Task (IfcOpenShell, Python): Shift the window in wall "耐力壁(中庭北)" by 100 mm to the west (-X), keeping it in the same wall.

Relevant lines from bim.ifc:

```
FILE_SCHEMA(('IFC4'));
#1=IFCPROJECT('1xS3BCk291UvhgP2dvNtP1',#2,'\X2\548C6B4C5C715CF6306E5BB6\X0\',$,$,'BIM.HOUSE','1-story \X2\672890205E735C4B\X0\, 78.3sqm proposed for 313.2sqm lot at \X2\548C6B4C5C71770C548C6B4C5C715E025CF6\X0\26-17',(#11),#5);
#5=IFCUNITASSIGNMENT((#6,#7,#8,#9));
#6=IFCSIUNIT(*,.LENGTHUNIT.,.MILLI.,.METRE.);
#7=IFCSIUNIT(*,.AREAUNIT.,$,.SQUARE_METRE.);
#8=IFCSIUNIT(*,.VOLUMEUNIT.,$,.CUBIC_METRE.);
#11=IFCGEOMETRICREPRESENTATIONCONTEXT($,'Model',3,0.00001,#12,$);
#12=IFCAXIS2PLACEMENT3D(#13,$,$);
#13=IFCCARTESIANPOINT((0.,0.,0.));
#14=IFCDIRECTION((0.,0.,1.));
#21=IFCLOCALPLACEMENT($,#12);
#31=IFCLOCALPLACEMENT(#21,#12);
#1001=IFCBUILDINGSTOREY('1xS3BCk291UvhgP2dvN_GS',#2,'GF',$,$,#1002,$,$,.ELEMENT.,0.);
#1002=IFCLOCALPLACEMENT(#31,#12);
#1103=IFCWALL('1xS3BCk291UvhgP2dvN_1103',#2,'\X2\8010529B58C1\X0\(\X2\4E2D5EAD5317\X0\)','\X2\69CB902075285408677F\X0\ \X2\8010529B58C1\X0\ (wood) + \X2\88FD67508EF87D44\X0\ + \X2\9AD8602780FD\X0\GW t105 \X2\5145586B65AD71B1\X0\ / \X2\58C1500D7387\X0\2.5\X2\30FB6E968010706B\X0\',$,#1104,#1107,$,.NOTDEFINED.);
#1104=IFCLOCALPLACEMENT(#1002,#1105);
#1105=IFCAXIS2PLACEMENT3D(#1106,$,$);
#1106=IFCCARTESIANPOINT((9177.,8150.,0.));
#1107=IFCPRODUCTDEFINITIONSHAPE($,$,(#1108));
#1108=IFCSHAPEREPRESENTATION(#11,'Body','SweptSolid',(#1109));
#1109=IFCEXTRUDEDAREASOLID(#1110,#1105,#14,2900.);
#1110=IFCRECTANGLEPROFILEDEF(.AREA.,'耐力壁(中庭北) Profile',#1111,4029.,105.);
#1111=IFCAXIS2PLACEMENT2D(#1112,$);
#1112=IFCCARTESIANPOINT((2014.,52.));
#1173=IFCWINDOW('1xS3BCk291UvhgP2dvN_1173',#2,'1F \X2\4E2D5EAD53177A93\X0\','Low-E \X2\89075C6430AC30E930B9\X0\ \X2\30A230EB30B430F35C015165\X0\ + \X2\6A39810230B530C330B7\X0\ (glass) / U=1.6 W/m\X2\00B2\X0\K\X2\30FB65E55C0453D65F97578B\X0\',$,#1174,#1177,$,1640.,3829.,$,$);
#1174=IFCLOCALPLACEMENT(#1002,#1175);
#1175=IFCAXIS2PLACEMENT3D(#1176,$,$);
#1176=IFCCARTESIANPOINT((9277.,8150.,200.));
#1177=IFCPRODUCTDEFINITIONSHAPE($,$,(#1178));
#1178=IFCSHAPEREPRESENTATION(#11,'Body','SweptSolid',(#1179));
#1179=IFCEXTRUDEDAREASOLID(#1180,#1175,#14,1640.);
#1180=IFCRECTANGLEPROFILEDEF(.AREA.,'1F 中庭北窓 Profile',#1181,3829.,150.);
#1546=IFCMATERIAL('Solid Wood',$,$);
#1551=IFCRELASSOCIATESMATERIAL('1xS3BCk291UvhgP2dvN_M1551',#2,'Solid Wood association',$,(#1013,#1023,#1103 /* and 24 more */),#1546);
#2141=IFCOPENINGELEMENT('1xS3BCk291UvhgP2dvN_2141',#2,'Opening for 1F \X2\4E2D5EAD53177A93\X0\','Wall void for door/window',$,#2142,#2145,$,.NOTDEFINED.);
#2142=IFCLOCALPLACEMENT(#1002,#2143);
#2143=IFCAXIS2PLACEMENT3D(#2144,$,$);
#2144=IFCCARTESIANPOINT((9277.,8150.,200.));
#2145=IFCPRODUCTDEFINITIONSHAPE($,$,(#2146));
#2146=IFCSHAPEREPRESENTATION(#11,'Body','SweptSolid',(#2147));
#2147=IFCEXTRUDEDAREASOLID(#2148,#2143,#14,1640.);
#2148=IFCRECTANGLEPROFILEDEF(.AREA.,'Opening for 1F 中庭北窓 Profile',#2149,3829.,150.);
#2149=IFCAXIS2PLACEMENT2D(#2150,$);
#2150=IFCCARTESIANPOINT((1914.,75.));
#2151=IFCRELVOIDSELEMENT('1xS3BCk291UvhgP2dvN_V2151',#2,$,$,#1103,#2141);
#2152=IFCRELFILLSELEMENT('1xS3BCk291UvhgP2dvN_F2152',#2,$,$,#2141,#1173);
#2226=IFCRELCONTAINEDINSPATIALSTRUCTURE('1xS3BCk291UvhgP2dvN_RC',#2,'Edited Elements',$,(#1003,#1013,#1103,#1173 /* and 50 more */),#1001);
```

```python
import ifcopenshell
import ifcopenshell.api.geometry
import ifcopenshell.util.placement

model = ifcopenshell.open("bim.ifc")

window = model.by_guid("1xS3BCk291UvhgP2dvN_1173")
opening = window.FillsVoids[0].RelatingOpeningElement
wall = opening.VoidsElements[0].RelatingBuildingElement

wall_matrix = ifcopenshell.util.placement.get_local_placement(wall.ObjectPlacement)
shift = wall_matrix[:3, 0] * -100.0
before = ifcopenshell.util.placement.get_local_placement(window.ObjectPlacement)[:3, 3].copy()

# The window is not placed relative to its opening, so move both.
for product in (opening, window):
    matrix = ifcopenshell.util.placement.get_local_placement(product.ObjectPlacement)
    matrix[:3, 3] += shift
    ifcopenshell.api.geometry.edit_object_placement(model, product=product, matrix=matrix, is_si=False)

after = ifcopenshell.util.placement.get_local_placement(window.ObjectPlacement)[:3, 3]
print("window moved by", (after - before).round(3) + 0.0)

model.write("bim_v2.ifc")
```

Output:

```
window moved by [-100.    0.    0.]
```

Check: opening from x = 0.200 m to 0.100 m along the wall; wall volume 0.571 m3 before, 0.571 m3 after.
